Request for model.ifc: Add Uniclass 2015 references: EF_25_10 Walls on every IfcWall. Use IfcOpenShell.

First a look at what the model holds.

```python
import ifcopenshell

model = ifcopenshell.open("model.ifc")
print(model.schema)
print("classifications:", [c.Name for c in model.by_type("IfcClassification")])
for ifc_class in ("IfcDoor", "IfcRoof", "IfcStair", "IfcWall", "IfcWindow"):
    print(ifc_class, len(model.by_type(ifc_class)))
```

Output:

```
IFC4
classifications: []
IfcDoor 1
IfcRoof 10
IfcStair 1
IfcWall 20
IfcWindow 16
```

```python
import ifcopenshell
import ifcopenshell.api.classification

model = ifcopenshell.open("model.ifc")

system = ifcopenshell.api.classification.add_classification(model, classification="Uniclass 2015")

codes = {
    "IfcWall": ("EF_25_10", "Walls"),
}
for ifc_class, (code, name) in codes.items():
    products = model.by_type(ifc_class)
    ifcopenshell.api.classification.add_reference(
        model, products=products, classification=system, identification=code, name=name
    )
    print(code, len(products))

model.write("model_updated.ifc")
```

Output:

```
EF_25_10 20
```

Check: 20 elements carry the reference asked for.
